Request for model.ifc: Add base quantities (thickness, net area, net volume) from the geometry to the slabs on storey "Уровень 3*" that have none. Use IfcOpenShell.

First a look at what the model holds.

```python
import ifcopenshell
import ifcopenshell.util.element
import ifcopenshell.util.unit

model = ifcopenshell.open("model.ifc")
print(model.schema)
for unit_type in ("LENGTHUNIT", "AREAUNIT", "VOLUMEUNIT"):
    print(unit_type, ifcopenshell.util.unit.calculate_unit_scale(model, unit_type))
storey = next(s for s in model.by_type("IfcBuildingStorey") if s.Name == "Уровень 3*")
slabs = [e for e in ifcopenshell.util.element.get_decomposition(storey) if e.is_a("IfcSlab")]
for e in sorted(slabs, key=lambda e: e.id()):
    print(e.id(), e.is_a(), e.Name, list(ifcopenshell.util.element.get_psets(e, qtos_only=True)), sep=" | ")
```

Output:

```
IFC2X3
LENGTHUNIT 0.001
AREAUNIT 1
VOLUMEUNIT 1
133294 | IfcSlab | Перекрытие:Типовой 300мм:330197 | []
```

```python
import ifcopenshell
import ifcopenshell.api.pset
import ifcopenshell.geom
import ifcopenshell.util.element
import ifcopenshell.util.shape
import ifcopenshell.util.unit

model = ifcopenshell.open("model.ifc")
unit_scale = ifcopenshell.util.unit.calculate_unit_scale(model)
area_scale = ifcopenshell.util.unit.calculate_unit_scale(model, "AREAUNIT")
volume_scale = ifcopenshell.util.unit.calculate_unit_scale(model, "VOLUMEUNIT")
settings = ifcopenshell.geom.settings()

storey = next(s for s in model.by_type("IfcBuildingStorey") if s.Name == "Уровень 3*")
slabs = [e for e in ifcopenshell.util.element.get_decomposition(storey) if e.is_a("IfcSlab")]

for e in sorted(slabs, key=lambda e: e.id()):
    if ifcopenshell.util.element.get_psets(e, qtos_only=True, should_inherit=False):
        continue
    # Geometry comes back in metres, in the element's own axes.
    shape = ifcopenshell.geom.create_shape(settings, e)
    values = {
        "Width": ifcopenshell.util.shape.get_z(shape.geometry) / unit_scale,
        "NetArea": ifcopenshell.util.shape.get_footprint_area(shape.geometry) / area_scale,
        "NetVolume": ifcopenshell.util.shape.get_volume(shape.geometry) / volume_scale,
    }
    qto = ifcopenshell.api.pset.add_qto(model, product=e, name="BaseQuantities")
    ifcopenshell.api.pset.edit_qto(model, qto=qto, properties=values)
    print(e.id(), {k: round(v, 3) for k, v in values.items()})

model.write("model_v2.ifc")
```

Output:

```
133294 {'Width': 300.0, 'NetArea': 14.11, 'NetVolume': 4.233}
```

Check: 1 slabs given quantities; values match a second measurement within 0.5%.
